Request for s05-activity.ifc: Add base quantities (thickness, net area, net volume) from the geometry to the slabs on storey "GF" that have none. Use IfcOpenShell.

First a look at what the model holds.

```python
import ifcopenshell
import ifcopenshell.util.element
import ifcopenshell.util.unit

model = ifcopenshell.open("s05-activity.ifc")
print(model.schema)
for unit_type in ("LENGTHUNIT", "AREAUNIT", "VOLUMEUNIT"):
    print(unit_type, ifcopenshell.util.unit.calculate_unit_scale(model, unit_type))
storey = next(s for s in model.by_type("IfcBuildingStorey") if s.Name == "GF")
slabs = [e for e in ifcopenshell.util.element.get_decomposition(storey) if e.is_a("IfcSlab")]
for e in sorted(slabs, key=lambda e: e.id()):
    print(e.id(), e.is_a(), e.Name, list(ifcopenshell.util.element.get_psets(e, qtos_only=True)), sep=" | ")
```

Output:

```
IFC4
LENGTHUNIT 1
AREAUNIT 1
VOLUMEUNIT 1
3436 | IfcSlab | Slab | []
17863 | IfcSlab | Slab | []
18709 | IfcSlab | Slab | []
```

```python
import ifcopenshell
import ifcopenshell.api.pset
import ifcopenshell.geom
import ifcopenshell.util.element
import ifcopenshell.util.shape
import ifcopenshell.util.unit

model = ifcopenshell.open("s05-activity.ifc")
unit_scale = ifcopenshell.util.unit.calculate_unit_scale(model)
area_scale = ifcopenshell.util.unit.calculate_unit_scale(model, "AREAUNIT")
volume_scale = ifcopenshell.util.unit.calculate_unit_scale(model, "VOLUMEUNIT")
settings = ifcopenshell.geom.settings()

storey = next(s for s in model.by_type("IfcBuildingStorey") if s.Name == "GF")
slabs = [e for e in ifcopenshell.util.element.get_decomposition(storey) if e.is_a("IfcSlab")]

for e in sorted(slabs, key=lambda e: e.id()):
    if ifcopenshell.util.element.get_psets(e, qtos_only=True, should_inherit=False):
        continue
    # Geometry comes back in metres, in the element's own axes.
    shape = ifcopenshell.geom.create_shape(settings, e)
    values = {
        "Width": ifcopenshell.util.shape.get_z(shape.geometry) / unit_scale,
        "NetArea": ifcopenshell.util.shape.get_footprint_area(shape.geometry) / area_scale,
        "NetVolume": ifcopenshell.util.shape.get_volume(shape.geometry) / volume_scale,
    }
    qto = ifcopenshell.api.pset.add_qto(model, product=e, name="Qto_SlabBaseQuantities")
    ifcopenshell.api.pset.edit_qto(model, qto=qto, properties=values)
    print(e.id(), {k: round(v, 3) for k, v in values.items()})

model.write("s05-activity_v2.ifc")
```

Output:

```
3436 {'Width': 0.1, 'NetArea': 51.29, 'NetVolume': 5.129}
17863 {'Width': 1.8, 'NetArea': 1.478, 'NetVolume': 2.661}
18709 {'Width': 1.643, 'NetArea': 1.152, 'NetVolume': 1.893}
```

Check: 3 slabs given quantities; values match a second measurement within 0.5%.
